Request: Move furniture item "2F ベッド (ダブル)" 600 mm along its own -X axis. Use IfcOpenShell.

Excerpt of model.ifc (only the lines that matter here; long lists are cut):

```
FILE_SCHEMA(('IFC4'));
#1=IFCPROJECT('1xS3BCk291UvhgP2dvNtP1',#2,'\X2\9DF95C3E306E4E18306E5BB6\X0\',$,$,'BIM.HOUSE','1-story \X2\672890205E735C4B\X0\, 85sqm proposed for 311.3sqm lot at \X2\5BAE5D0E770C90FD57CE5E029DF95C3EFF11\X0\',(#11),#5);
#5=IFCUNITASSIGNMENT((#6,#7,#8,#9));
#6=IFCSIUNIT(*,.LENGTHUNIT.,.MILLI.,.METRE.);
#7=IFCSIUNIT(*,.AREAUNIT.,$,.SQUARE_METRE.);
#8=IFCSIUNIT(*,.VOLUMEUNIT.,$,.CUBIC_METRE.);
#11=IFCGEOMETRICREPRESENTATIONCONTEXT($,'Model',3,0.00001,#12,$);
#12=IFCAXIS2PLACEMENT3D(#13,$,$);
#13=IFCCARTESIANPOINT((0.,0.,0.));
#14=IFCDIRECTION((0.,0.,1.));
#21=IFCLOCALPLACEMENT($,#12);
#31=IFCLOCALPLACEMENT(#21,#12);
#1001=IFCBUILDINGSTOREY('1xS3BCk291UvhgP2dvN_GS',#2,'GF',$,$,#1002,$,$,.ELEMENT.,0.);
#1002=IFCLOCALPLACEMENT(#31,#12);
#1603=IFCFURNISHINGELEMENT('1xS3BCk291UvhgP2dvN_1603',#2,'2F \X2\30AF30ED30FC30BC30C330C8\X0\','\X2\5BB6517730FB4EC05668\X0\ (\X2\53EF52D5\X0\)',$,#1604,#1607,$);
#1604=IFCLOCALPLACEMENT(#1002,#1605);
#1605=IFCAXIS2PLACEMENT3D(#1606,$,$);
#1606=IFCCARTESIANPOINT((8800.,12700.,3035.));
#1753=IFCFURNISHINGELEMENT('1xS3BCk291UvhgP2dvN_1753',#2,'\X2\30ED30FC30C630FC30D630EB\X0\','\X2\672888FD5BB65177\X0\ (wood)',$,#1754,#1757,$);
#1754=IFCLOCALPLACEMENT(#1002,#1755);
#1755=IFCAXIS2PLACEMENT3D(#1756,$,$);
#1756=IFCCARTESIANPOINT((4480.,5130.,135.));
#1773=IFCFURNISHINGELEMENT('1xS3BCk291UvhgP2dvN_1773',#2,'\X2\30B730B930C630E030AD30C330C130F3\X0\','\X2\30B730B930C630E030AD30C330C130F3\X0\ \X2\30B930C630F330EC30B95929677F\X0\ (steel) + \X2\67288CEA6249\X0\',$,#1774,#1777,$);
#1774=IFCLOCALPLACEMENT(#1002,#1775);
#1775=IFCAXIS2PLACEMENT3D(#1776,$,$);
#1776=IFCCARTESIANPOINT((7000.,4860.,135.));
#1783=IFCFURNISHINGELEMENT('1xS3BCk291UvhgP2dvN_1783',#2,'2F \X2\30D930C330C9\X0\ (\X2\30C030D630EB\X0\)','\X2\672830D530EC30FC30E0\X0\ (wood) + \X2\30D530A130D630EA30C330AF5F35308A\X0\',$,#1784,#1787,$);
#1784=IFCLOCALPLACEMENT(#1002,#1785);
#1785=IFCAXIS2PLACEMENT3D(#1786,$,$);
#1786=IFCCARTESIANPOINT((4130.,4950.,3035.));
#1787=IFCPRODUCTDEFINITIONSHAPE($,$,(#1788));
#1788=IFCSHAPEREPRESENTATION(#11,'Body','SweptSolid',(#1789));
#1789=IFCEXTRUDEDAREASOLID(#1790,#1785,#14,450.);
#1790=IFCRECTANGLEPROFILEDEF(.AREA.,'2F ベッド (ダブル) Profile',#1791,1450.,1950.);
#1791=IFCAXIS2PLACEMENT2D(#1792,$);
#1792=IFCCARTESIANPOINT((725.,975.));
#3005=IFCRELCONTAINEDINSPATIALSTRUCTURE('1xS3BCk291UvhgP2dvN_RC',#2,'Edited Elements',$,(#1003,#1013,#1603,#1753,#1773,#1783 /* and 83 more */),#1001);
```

```python
import ifcopenshell
import ifcopenshell.api.geometry
import ifcopenshell.util.placement
import ifcopenshell.util.unit

model = ifcopenshell.open("model.ifc")
unit_scale = ifcopenshell.util.unit.calculate_unit_scale(model)

item = model.by_guid("1xS3BCk291UvhgP2dvN_1783")
matrix = ifcopenshell.util.placement.get_local_placement(item.ObjectPlacement)
matrix[:3, 3] -= matrix[:3, 0] * 0.6 / unit_scale
ifcopenshell.api.geometry.edit_object_placement(model, product=item, matrix=matrix, is_si=False)

print(ifcopenshell.util.placement.get_local_placement(item.ObjectPlacement).round(3) + 0.0)

model.write("model_rev.ifc")
```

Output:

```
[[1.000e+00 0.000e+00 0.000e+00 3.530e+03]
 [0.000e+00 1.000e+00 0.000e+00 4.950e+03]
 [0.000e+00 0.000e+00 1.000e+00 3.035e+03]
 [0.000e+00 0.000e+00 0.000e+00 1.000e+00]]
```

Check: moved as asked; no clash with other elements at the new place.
